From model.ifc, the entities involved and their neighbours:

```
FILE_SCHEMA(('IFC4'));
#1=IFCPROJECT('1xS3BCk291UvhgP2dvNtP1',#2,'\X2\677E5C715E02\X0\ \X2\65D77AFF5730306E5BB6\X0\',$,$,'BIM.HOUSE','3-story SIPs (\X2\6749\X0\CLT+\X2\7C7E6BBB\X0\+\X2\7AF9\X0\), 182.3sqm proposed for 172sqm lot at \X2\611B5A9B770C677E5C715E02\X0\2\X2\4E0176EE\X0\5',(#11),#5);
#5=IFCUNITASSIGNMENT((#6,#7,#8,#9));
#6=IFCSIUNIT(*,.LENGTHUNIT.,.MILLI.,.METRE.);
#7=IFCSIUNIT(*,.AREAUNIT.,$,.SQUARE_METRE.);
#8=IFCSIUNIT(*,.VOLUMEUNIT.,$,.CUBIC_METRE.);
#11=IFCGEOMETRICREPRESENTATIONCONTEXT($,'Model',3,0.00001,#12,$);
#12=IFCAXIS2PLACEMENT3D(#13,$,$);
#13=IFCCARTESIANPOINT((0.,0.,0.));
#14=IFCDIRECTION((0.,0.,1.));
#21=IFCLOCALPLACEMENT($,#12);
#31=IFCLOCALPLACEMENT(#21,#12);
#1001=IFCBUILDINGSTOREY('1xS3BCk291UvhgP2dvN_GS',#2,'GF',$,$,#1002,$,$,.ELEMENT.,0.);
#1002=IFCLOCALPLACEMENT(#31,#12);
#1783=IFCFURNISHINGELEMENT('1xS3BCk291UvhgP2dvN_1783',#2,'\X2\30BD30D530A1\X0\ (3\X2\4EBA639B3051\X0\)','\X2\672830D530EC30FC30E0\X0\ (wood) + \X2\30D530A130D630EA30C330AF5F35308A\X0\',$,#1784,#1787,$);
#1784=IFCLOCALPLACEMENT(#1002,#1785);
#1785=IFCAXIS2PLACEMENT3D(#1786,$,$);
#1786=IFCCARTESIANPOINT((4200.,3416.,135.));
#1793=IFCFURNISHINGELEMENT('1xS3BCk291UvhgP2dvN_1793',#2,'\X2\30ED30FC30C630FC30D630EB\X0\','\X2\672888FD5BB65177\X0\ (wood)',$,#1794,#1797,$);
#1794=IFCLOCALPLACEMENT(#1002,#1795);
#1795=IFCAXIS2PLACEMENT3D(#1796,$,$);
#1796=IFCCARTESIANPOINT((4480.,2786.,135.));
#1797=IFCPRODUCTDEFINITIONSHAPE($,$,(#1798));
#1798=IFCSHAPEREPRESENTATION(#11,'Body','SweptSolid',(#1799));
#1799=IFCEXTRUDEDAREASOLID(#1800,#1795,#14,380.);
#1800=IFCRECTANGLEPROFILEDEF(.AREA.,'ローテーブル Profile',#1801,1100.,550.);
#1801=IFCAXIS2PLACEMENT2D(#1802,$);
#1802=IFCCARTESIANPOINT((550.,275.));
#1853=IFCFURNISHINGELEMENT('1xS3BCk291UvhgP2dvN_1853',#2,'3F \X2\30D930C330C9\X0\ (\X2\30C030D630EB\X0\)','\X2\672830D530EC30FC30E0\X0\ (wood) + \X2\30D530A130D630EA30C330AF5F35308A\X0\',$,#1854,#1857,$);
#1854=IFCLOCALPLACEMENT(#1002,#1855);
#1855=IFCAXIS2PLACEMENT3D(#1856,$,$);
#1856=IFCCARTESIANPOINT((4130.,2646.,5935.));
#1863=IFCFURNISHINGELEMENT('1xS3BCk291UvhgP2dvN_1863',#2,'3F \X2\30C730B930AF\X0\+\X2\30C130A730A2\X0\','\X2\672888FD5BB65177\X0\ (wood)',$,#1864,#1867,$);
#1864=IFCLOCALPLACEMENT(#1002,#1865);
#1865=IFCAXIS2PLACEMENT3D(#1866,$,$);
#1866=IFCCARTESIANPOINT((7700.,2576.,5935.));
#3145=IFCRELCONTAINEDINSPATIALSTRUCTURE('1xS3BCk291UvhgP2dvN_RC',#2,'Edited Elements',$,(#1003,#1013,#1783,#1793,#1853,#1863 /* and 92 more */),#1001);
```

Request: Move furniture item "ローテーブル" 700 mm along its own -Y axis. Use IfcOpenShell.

```python
import ifcopenshell
import ifcopenshell.api.geometry
import ifcopenshell.util.placement

model = ifcopenshell.open("model.ifc")

item = model.by_id(1793)
matrix = ifcopenshell.util.placement.get_local_placement(item.ObjectPlacement)
matrix[:3, 3] -= matrix[:3, 1] * 700.0
ifcopenshell.api.geometry.edit_object_placement(model, product=item, matrix=matrix, is_si=False)

print(ifcopenshell.util.placement.get_local_placement(item.ObjectPlacement).round(3) + 0.0)

model.write("model_v2.ifc")
```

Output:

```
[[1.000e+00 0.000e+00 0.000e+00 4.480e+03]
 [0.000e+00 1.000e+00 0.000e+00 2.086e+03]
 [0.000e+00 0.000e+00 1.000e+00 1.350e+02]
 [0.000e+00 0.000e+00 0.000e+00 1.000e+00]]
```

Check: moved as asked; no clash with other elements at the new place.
